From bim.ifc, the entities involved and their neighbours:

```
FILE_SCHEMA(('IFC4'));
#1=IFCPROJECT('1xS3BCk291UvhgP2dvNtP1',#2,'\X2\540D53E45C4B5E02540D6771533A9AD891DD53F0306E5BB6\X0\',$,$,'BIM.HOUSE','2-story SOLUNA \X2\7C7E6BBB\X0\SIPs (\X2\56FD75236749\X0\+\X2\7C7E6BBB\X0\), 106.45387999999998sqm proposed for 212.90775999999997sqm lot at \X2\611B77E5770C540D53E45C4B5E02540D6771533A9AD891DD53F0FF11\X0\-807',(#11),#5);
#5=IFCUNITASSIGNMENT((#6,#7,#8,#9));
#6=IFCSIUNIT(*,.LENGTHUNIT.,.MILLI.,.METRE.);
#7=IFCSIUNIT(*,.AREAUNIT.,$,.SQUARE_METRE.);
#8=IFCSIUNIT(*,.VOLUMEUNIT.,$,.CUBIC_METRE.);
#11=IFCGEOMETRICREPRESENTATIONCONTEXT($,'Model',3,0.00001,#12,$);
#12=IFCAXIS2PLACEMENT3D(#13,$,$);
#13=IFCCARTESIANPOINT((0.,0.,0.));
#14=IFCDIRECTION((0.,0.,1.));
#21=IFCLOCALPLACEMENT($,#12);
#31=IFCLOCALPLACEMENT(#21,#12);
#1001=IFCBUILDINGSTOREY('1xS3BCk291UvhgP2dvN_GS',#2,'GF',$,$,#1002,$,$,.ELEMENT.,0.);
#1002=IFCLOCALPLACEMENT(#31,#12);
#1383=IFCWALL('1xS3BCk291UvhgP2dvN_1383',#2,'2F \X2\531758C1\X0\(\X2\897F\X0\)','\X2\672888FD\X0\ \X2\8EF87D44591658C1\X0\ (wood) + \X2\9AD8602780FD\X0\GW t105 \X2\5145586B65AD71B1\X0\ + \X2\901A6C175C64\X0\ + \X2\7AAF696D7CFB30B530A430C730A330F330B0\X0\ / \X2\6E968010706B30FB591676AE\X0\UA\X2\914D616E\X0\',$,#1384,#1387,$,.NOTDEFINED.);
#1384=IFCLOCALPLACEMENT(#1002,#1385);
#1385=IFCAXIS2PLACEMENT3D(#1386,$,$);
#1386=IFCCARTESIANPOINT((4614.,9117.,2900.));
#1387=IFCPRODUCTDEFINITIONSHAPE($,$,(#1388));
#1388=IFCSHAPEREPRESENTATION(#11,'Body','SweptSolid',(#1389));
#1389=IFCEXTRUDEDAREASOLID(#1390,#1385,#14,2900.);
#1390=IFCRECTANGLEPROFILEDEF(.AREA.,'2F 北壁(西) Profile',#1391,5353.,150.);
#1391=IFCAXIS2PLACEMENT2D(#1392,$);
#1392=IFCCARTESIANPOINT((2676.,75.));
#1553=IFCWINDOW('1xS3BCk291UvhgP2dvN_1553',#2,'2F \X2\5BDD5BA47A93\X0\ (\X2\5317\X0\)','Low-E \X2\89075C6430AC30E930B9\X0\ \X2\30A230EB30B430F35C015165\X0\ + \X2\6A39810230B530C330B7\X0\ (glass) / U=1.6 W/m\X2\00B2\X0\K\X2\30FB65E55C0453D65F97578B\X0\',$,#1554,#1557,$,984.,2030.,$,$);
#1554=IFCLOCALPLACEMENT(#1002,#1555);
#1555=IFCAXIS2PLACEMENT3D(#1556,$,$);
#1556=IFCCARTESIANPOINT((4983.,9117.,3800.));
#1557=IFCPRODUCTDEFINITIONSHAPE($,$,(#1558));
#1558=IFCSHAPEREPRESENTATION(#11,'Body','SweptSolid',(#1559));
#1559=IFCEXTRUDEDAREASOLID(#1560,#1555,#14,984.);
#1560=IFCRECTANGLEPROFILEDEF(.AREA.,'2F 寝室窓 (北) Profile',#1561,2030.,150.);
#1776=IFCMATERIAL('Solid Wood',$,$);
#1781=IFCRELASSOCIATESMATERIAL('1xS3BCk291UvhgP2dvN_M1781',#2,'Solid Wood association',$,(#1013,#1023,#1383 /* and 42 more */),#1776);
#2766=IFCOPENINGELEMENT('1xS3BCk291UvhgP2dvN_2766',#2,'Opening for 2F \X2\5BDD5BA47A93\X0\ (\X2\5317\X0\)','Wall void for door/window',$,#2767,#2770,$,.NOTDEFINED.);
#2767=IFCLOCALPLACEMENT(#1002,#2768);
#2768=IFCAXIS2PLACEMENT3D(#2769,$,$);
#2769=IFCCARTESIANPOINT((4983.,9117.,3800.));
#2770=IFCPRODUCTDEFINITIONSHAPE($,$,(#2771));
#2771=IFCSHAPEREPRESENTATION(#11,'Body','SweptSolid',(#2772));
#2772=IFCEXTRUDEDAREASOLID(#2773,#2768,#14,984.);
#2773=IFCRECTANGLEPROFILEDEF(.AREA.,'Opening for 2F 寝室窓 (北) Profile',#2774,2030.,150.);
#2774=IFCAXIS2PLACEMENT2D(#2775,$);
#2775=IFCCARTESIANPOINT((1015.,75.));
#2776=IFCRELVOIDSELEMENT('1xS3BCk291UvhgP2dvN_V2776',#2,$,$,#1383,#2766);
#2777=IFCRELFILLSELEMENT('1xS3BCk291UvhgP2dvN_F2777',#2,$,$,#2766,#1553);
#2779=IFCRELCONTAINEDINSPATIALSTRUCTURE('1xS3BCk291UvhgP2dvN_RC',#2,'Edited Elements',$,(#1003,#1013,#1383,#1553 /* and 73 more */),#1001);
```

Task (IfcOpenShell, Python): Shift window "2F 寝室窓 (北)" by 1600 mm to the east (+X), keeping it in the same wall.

```python
import ifcopenshell
import ifcopenshell.api.geometry
import ifcopenshell.util.placement

model = ifcopenshell.open("bim.ifc")

window = model.by_guid("1xS3BCk291UvhgP2dvN_1553")
opening = window.FillsVoids[0].RelatingOpeningElement
wall = opening.VoidsElements[0].RelatingBuildingElement

wall_matrix = ifcopenshell.util.placement.get_local_placement(wall.ObjectPlacement)
shift = wall_matrix[:3, 0] * 1600.0
before = ifcopenshell.util.placement.get_local_placement(window.ObjectPlacement)[:3, 3].copy()

# The window is not placed relative to its opening, so move both.
for product in (opening, window):
    matrix = ifcopenshell.util.placement.get_local_placement(product.ObjectPlacement)
    matrix[:3, 3] += shift
    ifcopenshell.api.geometry.edit_object_placement(model, product=product, matrix=matrix, is_si=False)

after = ifcopenshell.util.placement.get_local_placement(window.ObjectPlacement)[:3, 3]
print("window moved by", (after - before).round(3) + 0.0)

model.write("bim_rev.ifc")
```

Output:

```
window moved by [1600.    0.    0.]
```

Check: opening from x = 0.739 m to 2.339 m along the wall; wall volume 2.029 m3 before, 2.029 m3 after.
